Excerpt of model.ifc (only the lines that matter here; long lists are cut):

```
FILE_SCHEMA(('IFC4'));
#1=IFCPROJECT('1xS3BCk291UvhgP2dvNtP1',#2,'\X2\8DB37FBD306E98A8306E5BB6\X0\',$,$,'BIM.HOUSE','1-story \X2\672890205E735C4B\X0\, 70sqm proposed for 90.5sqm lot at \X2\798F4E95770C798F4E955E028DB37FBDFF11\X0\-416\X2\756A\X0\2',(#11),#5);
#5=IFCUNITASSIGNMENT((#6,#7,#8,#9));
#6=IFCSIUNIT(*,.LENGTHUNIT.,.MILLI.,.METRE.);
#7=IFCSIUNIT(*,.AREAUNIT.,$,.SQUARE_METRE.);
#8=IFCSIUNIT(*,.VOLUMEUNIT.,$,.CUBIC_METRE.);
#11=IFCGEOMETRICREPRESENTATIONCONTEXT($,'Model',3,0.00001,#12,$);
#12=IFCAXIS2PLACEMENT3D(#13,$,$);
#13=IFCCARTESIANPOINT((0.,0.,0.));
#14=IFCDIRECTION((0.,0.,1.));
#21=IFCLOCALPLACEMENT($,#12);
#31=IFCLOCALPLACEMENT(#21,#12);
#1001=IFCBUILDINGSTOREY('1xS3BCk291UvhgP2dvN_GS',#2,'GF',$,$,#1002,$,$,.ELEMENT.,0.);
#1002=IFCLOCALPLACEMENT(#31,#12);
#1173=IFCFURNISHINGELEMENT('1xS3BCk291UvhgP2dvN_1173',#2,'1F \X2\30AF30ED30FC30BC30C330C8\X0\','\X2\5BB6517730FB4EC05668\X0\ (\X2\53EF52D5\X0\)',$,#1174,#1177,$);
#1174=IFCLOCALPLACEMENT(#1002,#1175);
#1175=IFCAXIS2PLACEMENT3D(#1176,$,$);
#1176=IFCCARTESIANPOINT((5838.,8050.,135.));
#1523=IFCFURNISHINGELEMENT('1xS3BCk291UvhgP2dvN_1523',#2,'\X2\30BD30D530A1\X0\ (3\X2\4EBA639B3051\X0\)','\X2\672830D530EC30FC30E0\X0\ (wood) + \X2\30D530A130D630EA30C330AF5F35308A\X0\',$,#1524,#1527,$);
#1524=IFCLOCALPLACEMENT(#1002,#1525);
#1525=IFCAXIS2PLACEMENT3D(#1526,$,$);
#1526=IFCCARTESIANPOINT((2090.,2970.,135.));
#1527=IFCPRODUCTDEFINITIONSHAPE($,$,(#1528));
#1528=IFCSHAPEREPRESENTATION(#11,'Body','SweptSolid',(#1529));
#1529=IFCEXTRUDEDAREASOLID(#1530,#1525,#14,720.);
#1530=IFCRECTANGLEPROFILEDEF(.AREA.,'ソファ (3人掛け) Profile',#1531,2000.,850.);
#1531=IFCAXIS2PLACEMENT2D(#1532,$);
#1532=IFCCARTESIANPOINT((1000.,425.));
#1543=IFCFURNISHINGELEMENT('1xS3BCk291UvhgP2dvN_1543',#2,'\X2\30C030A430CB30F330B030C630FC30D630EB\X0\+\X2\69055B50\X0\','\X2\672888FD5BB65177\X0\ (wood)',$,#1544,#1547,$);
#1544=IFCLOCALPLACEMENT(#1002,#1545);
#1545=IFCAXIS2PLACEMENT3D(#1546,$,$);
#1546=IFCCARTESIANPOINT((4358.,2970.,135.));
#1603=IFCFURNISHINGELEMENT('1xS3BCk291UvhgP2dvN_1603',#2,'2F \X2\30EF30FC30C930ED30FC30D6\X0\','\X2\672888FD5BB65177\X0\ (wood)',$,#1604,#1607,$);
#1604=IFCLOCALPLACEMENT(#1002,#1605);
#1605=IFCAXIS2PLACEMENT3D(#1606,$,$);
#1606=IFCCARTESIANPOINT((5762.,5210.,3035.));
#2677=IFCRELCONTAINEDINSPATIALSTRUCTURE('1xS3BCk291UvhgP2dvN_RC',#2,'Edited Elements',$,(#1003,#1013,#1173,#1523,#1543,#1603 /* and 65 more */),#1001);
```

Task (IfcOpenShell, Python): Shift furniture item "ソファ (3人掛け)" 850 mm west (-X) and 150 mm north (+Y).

```python
import ifcopenshell
import ifcopenshell.api.geometry
import ifcopenshell.util.placement
import ifcopenshell.util.unit

model = ifcopenshell.open("model.ifc")
unit_scale = ifcopenshell.util.unit.calculate_unit_scale(model)

item = model.by_guid("1xS3BCk291UvhgP2dvN_1523")
matrix = ifcopenshell.util.placement.get_local_placement(item.ObjectPlacement)
matrix[0, 3] -= 0.85 / unit_scale
matrix[1, 3] += 0.15 / unit_scale
ifcopenshell.api.geometry.edit_object_placement(model, product=item, matrix=matrix, is_si=False)

print(ifcopenshell.util.placement.get_local_placement(item.ObjectPlacement).round(3) + 0.0)

model.write("model_rev.ifc")
```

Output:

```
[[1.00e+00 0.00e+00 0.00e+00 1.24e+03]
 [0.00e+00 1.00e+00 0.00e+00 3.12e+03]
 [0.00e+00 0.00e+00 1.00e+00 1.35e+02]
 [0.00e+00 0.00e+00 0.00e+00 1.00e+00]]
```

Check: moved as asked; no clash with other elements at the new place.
